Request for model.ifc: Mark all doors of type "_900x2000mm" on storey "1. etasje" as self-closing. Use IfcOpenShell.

First a look at what the model holds.

```python
import ifcopenshell
import ifcopenshell.util.element

model = ifcopenshell.open("model.ifc")
print(model.schema)
storey = next(s for s in model.by_type("IfcBuildingStorey") if s.Name == "1. etasje")
doors = [e for e in ifcopenshell.util.element.get_decomposition(storey) if e.is_a("IfcDoor")]
seen = {}
for e in doors:
    element_type = ifcopenshell.util.element.get_type(e)
    key = (element_type.Name if element_type != e and element_type else None, ifcopenshell.util.element.get_pset(e, "Pset_DoorCommon", "SelfClosing"))
    seen[key] = seen.get(key, 0) + 1
for (name, value), count in sorted(seen.items(), key=str):
    print(count, "x", name, "|", value)
```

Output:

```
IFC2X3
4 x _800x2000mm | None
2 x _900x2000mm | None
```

```python
import ifcopenshell
import ifcopenshell.api.pset
import ifcopenshell.util.element

model = ifcopenshell.open("model.ifc")

storey = next(s for s in model.by_type("IfcBuildingStorey") if s.Name == "1. etasje")
doors = [e for e in ifcopenshell.util.element.get_decomposition(storey) if e.is_a("IfcDoor")]

count = 0
for e in doors:
    element_type = ifcopenshell.util.element.get_type(e)
    if element_type in (None, e) or element_type.Name != "_900x2000mm":
        continue
    # add_pset returns the element's existing set when there is one.
    pset = ifcopenshell.api.pset.add_pset(model, product=e, name="Pset_DoorCommon")
    ifcopenshell.api.pset.edit_pset(model, pset=pset, properties={"SelfClosing": True})
    count += 1

print(count, "doors updated")

model.write("model_updated.ifc")
```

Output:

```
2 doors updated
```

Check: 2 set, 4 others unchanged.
